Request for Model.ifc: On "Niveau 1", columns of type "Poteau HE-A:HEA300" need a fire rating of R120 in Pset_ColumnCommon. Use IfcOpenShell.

First a look at what the model holds.

```python
import ifcopenshell
import ifcopenshell.util.element

model = ifcopenshell.open("Model.ifc")
print(model.schema)
storey = next(s for s in model.by_type("IfcBuildingStorey") if s.Name == "Niveau 1")
columns = [e for e in ifcopenshell.util.element.get_decomposition(storey) if e.is_a("IfcColumn")]
seen = {}
for e in columns:
    element_type = ifcopenshell.util.element.get_type(e)
    key = (element_type.Name if element_type != e and element_type else None, ifcopenshell.util.element.get_pset(e, "Pset_ColumnCommon", "FireRating"))
    seen[key] = seen.get(key, 0) + 1
for (name, value), count in sorted(seen.items(), key=str):
    print(count, "x", name, "|", value)
```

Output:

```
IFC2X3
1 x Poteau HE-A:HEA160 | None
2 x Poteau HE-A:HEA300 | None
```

```python
import ifcopenshell
import ifcopenshell.api.pset
import ifcopenshell.util.element

model = ifcopenshell.open("Model.ifc")

storey = next(s for s in model.by_type("IfcBuildingStorey") if s.Name == "Niveau 1")
columns = [e for e in ifcopenshell.util.element.get_decomposition(storey) if e.is_a("IfcColumn")]

count = 0
for e in columns:
    element_type = ifcopenshell.util.element.get_type(e)
    if element_type in (None, e) or element_type.Name != "Poteau HE-A:HEA300":
        continue
    # add_pset returns the element's existing set when there is one.
    pset = ifcopenshell.api.pset.add_pset(model, product=e, name="Pset_ColumnCommon")
    ifcopenshell.api.pset.edit_pset(model, pset=pset, properties={"FireRating": "R120"})
    count += 1

print(count, "columns updated")

model.write("Model_v2.ifc")
```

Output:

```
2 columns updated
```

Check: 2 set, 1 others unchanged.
